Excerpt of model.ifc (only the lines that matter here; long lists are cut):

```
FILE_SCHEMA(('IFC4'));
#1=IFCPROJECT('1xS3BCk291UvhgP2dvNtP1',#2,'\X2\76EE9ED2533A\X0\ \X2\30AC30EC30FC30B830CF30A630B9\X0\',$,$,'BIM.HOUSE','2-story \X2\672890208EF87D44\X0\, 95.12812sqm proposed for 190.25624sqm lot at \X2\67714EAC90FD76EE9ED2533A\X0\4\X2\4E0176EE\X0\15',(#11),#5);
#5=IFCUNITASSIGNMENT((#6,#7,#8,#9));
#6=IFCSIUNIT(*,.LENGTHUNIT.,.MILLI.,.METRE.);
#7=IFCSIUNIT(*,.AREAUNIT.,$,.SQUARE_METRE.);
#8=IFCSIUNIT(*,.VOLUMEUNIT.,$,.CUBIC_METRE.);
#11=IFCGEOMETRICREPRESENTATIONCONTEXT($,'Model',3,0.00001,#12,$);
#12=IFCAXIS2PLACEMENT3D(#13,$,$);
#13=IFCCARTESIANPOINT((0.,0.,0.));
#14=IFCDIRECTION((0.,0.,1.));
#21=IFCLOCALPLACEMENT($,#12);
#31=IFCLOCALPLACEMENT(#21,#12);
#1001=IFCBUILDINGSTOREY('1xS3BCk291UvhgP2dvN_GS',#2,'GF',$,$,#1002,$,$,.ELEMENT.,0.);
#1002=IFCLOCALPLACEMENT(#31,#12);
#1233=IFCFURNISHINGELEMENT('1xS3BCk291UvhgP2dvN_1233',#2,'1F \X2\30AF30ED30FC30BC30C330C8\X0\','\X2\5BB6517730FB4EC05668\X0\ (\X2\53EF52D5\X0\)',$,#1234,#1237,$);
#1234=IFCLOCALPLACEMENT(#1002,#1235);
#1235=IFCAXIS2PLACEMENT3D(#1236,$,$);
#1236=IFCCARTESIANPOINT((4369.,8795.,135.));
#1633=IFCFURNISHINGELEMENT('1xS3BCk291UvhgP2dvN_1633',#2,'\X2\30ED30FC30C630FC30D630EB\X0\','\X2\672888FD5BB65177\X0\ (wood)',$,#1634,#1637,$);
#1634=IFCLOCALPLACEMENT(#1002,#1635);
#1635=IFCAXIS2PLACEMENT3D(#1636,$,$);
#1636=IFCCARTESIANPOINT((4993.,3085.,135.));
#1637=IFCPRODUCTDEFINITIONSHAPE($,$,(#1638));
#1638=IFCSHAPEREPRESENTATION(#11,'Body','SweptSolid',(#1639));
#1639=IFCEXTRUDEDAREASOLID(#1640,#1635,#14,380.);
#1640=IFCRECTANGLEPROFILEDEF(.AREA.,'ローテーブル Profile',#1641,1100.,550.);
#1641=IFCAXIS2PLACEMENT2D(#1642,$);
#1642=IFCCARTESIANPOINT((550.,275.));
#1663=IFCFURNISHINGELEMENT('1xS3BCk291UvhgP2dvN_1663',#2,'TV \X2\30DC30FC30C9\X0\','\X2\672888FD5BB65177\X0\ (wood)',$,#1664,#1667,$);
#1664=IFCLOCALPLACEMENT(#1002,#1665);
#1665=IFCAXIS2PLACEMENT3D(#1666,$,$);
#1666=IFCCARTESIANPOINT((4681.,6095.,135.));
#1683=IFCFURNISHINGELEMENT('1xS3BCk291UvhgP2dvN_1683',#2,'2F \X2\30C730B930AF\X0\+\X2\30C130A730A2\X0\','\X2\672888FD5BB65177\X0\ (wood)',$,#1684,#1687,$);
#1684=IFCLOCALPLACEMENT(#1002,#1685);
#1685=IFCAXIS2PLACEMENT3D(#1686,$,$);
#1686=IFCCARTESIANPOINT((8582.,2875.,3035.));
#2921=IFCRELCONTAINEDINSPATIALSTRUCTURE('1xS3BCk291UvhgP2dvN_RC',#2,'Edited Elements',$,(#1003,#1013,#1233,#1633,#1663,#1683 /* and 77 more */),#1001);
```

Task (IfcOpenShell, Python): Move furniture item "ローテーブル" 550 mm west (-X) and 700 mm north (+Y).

```python
import ifcopenshell
import ifcopenshell.api.geometry
import ifcopenshell.util.placement

model = ifcopenshell.open("model.ifc")

item = model.by_guid("1xS3BCk291UvhgP2dvN_1633")
matrix = ifcopenshell.util.placement.get_local_placement(item.ObjectPlacement)
matrix[0, 3] -= 550.0
matrix[1, 3] += 700.0
ifcopenshell.api.geometry.edit_object_placement(model, product=item, matrix=matrix, is_si=False)

print(ifcopenshell.util.placement.get_local_placement(item.ObjectPlacement).round(3) + 0.0)

model.write("model-out.ifc")
```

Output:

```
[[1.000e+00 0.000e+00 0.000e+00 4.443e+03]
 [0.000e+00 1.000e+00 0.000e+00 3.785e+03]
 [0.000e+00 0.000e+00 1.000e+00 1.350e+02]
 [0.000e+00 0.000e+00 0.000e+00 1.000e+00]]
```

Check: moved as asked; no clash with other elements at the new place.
